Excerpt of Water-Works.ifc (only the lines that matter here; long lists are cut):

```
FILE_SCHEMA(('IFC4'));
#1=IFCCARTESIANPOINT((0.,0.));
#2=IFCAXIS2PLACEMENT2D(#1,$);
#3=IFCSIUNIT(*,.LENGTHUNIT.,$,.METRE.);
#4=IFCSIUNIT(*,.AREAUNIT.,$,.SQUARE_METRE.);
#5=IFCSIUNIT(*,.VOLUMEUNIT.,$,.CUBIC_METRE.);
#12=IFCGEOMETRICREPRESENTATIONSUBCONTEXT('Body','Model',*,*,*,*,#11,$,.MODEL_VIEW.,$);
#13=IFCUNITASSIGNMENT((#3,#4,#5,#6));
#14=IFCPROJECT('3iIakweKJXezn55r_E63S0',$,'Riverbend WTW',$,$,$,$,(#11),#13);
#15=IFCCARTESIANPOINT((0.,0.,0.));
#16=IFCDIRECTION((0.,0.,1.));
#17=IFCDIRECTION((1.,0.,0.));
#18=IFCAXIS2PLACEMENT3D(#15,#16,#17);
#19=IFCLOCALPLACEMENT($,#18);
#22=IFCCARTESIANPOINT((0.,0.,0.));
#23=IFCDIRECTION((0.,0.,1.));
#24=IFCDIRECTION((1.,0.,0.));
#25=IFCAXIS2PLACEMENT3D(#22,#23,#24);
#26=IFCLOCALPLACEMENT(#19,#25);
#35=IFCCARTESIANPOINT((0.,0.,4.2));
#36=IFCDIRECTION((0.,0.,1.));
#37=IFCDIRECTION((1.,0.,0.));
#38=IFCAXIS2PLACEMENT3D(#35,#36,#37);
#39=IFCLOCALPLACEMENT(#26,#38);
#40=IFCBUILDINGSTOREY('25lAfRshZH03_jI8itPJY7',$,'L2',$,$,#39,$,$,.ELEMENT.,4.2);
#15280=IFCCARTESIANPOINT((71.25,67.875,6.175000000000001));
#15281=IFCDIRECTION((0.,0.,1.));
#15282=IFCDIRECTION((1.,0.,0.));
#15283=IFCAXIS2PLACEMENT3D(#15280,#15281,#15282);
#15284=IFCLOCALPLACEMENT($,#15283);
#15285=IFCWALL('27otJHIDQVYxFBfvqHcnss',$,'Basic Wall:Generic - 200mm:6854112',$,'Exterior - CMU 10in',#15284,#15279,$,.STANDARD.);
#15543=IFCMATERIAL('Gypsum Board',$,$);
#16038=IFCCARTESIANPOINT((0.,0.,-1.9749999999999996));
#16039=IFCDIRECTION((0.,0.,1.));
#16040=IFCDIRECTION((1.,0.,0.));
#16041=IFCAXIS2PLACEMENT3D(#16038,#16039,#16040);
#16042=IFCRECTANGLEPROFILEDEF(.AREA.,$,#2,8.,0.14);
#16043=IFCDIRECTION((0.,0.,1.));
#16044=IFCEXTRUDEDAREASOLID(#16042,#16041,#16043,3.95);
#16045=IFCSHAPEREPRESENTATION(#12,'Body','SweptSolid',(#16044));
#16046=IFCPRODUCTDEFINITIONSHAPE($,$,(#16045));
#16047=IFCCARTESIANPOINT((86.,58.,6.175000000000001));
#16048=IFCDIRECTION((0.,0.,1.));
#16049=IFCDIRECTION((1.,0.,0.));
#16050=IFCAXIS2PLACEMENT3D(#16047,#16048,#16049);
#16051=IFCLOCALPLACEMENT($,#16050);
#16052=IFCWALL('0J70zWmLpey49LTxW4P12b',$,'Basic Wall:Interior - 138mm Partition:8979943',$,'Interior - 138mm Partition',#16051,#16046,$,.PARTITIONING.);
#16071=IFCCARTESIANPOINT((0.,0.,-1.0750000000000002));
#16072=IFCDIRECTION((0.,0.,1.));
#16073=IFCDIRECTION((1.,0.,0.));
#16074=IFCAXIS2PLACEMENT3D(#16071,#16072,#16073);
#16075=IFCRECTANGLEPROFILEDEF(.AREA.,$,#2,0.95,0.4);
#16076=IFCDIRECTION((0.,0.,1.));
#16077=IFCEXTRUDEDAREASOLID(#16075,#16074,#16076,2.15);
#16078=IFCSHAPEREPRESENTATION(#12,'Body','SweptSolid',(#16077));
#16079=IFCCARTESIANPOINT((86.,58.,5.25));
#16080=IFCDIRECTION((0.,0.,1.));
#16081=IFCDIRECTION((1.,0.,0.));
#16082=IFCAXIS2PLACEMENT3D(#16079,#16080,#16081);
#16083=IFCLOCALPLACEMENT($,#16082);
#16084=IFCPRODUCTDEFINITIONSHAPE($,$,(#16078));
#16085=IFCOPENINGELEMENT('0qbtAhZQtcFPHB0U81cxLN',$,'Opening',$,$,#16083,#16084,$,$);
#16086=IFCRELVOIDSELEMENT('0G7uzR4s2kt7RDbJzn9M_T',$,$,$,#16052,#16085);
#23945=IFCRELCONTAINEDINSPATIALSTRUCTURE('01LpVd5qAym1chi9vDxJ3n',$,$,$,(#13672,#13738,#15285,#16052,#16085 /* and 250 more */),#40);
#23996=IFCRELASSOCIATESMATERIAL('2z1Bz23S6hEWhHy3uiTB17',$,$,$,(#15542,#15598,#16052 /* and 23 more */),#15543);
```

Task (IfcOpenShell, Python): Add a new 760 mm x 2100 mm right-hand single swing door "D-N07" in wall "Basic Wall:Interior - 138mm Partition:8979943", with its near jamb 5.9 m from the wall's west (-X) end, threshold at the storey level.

```python
import numpy as np
import ifcopenshell
import ifcopenshell.api.feature
import ifcopenshell.api.geometry
import ifcopenshell.api.root
import ifcopenshell.api.spatial
import ifcopenshell.geom
import ifcopenshell.util.element
import ifcopenshell.util.placement
import ifcopenshell.util.representation
import ifcopenshell.util.shape
import ifcopenshell.util.unit

model = ifcopenshell.open("Water-Works.ifc")
unit_scale = ifcopenshell.util.unit.calculate_unit_scale(model)
settings = ifcopenshell.geom.settings()


def volume(element):
    """Net volume in cubic metres, openings subtracted."""
    shape = ifcopenshell.geom.create_shape(settings, element)
    return ifcopenshell.util.shape.get_volume(shape.geometry)


wall = model.by_guid("0J70zWmLpey49LTxW4P12b")
storey = ifcopenshell.util.element.get_container(wall, ifc_class="IfcBuildingStorey")
context = ifcopenshell.util.representation.get_context(model, "Model", "Body", "MODEL_VIEW")
before = volume(wall)

width, height, from_end, sill = 0.76, 2.1, 5.9, 0.0  # metres

# The wall runs along its own X axis, and the end named is its -X end.
wall_shape = ifcopenshell.geom.create_shape(settings, wall)
x, y, z = ifcopenshell.util.shape.get_vertices(wall_shape.geometry).T
start = x.min() + from_end
face, thickness = float(y.min()), float(y.max() - y.min())
wall_matrix = ifcopenshell.util.placement.get_local_placement(wall.ObjectPlacement)
level = ifcopenshell.util.placement.get_local_placement(storey.ObjectPlacement)[2, 3]


def in_wall(x, y):
    """Placement at x, y metres in the wall's axes, at sill height."""
    matrix = wall_matrix.copy()
    matrix[:, 3] = wall_matrix @ np.array([x / unit_scale, y / unit_scale, 0.0, 1.0])
    matrix[2, 3] = level + sill / unit_scale
    return matrix


# Opening: a box that overshoots both wall faces by 50 mm.
opening = ifcopenshell.api.root.create_entity(model, ifc_class="IfcOpeningElement", predefined_type="OPENING")
box = ifcopenshell.api.geometry.add_wall_representation(
    model, context=context, length=width, height=height, thickness=thickness + 0.1
)
ifcopenshell.api.geometry.assign_representation(model, product=opening, representation=box)
ifcopenshell.api.geometry.edit_object_placement(model, product=opening, matrix=in_wall(start, face - 0.05), is_si=False)
ifcopenshell.api.feature.add_feature(model, feature=opening, element=wall)

door = ifcopenshell.api.root.create_entity(model, ifc_class="IfcDoor", name="D-N07", predefined_type="DOOR")
door.OverallWidth, door.OverallHeight = width / unit_scale, height / unit_scale
door.OperationType = "SINGLE_SWING_RIGHT"
body = ifcopenshell.api.geometry.add_door_representation(
    model,
    context=context,
    overall_width=door.OverallWidth,
    overall_height=door.OverallHeight,
    operation_type="SINGLE_SWING_RIGHT",
    lining_properties={"LiningDepth": thickness / unit_scale, "ThresholdDepth": thickness / unit_scale},
)
ifcopenshell.api.geometry.assign_representation(model, product=door, representation=body)
ifcopenshell.api.spatial.assign_container(model, products=[door], relating_structure=storey)
ifcopenshell.api.feature.add_filling(model, opening=opening, element=door)

# The lining spans the wall, so the door starts at the wall face.
ifcopenshell.api.geometry.edit_object_placement(model, product=door, matrix=in_wall(start, face), is_si=False)

after = volume(wall)

print(f"wall volume {before:.3f} -> {after:.3f} m3")

model.write("Water-Works_rev.ifc")
```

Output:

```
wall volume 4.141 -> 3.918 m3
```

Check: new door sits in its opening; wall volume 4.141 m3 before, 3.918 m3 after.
